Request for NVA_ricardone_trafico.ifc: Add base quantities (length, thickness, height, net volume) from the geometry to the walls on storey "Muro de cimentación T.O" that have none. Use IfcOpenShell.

First a look at what the model holds.

```python
import ifcopenshell
import ifcopenshell.util.element
import ifcopenshell.util.unit

model = ifcopenshell.open("NVA_ricardone_trafico.ifc")
print(model.schema)
for unit_type in ("LENGTHUNIT", "AREAUNIT", "VOLUMEUNIT"):
    print(unit_type, ifcopenshell.util.unit.calculate_unit_scale(model, unit_type))
storey = next(s for s in model.by_type("IfcBuildingStorey") if s.Name == "Muro de cimentación T.O")
walls = [e for e in ifcopenshell.util.element.get_decomposition(storey) if e.is_a("IfcWall")]
for e in sorted(walls, key=lambda e: e.id()):
    print(e.id(), e.is_a(), e.Name, list(ifcopenshell.util.element.get_psets(e, qtos_only=True)), sep=" | ")
```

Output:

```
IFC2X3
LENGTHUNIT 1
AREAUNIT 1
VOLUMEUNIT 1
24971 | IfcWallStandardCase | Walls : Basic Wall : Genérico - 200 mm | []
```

```python
import ifcopenshell
import ifcopenshell.api.pset
import ifcopenshell.geom
import ifcopenshell.util.element
import ifcopenshell.util.shape
import ifcopenshell.util.unit

model = ifcopenshell.open("NVA_ricardone_trafico.ifc")
unit_scale = ifcopenshell.util.unit.calculate_unit_scale(model)
volume_scale = ifcopenshell.util.unit.calculate_unit_scale(model, "VOLUMEUNIT")
settings = ifcopenshell.geom.settings()

storey = next(s for s in model.by_type("IfcBuildingStorey") if s.Name == "Muro de cimentación T.O")
walls = [e for e in ifcopenshell.util.element.get_decomposition(storey) if e.is_a("IfcWall")]

for e in sorted(walls, key=lambda e: e.id()):
    if ifcopenshell.util.element.get_psets(e, qtos_only=True, should_inherit=False):
        continue
    # Geometry comes back in metres, in the element's own axes.
    shape = ifcopenshell.geom.create_shape(settings, e)
    values = {
        "Length": ifcopenshell.util.shape.get_x(shape.geometry) / unit_scale,
        "Width": ifcopenshell.util.shape.get_y(shape.geometry) / unit_scale,
        "Height": ifcopenshell.util.shape.get_z(shape.geometry) / unit_scale,
        "NetVolume": ifcopenshell.util.shape.get_volume(shape.geometry) / volume_scale,
    }
    qto = ifcopenshell.api.pset.add_qto(model, product=e, name="BaseQuantities")
    ifcopenshell.api.pset.edit_qto(model, qto=qto, properties=values)
    print(e.id(), {k: round(v, 3) for k, v in values.items()})

model.write("NVA_ricardone_trafico_updated.ifc")
```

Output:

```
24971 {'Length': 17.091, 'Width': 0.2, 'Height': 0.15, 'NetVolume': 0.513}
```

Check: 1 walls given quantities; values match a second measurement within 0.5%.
